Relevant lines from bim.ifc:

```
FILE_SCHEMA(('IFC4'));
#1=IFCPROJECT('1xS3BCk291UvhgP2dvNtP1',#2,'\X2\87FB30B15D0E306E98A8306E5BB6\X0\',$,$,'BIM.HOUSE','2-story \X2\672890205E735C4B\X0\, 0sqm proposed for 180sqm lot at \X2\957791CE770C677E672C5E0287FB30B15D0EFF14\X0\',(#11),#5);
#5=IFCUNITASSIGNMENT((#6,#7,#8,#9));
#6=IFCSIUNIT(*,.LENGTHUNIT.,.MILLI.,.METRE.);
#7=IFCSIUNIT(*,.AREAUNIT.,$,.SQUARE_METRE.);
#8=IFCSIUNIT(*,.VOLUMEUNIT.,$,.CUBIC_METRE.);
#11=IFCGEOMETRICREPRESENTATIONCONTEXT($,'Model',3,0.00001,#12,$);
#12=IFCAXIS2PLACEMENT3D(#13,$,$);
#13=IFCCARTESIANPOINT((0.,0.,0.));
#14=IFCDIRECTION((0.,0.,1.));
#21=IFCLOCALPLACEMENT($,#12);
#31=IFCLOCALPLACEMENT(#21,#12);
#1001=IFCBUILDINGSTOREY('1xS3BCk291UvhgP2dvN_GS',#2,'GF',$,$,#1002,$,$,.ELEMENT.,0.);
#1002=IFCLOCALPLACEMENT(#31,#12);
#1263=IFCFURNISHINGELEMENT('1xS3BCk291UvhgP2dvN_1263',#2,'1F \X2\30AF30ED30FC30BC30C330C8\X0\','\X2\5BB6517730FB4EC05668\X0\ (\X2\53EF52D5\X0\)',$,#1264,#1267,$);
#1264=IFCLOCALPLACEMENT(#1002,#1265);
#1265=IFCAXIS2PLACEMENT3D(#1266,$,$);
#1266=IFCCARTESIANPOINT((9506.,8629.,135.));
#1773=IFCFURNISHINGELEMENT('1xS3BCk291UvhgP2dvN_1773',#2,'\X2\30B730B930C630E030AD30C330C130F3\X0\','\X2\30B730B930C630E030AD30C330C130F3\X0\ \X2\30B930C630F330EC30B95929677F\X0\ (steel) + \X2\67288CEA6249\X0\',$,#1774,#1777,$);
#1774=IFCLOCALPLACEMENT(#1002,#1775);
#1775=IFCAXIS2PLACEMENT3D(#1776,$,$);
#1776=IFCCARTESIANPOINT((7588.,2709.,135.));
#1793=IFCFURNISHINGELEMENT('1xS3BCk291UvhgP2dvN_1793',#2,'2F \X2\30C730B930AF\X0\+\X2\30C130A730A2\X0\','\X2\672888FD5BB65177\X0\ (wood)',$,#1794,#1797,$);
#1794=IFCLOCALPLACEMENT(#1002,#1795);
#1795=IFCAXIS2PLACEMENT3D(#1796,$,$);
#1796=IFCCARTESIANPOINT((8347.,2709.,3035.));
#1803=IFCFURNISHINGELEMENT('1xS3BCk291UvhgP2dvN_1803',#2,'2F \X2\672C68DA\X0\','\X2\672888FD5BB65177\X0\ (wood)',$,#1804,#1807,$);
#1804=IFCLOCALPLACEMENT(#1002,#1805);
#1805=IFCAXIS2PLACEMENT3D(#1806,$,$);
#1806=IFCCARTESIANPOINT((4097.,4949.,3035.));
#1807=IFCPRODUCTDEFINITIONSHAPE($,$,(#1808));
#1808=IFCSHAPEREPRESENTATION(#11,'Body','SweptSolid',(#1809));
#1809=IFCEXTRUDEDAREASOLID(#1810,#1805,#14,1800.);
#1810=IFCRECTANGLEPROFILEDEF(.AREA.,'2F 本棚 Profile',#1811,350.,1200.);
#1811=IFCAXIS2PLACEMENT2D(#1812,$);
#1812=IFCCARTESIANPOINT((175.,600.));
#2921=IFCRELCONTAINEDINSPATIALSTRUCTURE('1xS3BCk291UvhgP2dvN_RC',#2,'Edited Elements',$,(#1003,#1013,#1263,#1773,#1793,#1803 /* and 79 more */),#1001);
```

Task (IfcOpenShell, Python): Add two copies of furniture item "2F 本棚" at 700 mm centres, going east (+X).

```python
import numpy as np
import ifcopenshell
import ifcopenshell.api.geometry
import ifcopenshell.api.root
import ifcopenshell.util.element
import ifcopenshell.util.placement
import ifcopenshell.util.unit

model = ifcopenshell.open("bim.ifc")
unit_scale = ifcopenshell.util.unit.calculate_unit_scale(model)


def reuse_history(source, copy):
    """copy_class also copies each property set's owner history, people and application; keep the originals."""
    for rel in copy.IsDefinedBy:
        if rel.is_a("IfcRelDefinesByProperties") and (history := rel.RelatingPropertyDefinition.OwnerHistory):
            rel.RelatingPropertyDefinition.OwnerHistory = source.OwnerHistory
            ifcopenshell.util.element.remove_deep2(model, history)


source = model.by_guid("1xS3BCk291UvhgP2dvN_1803")
base = ifcopenshell.util.placement.get_local_placement(source.ObjectPlacement)
step = np.array([1.0, 0.0, 0.0]) * 0.7 / unit_scale

for i in range(1, 3):
    copy = ifcopenshell.api.root.copy_class(model, product=source)
    copy.Representation = ifcopenshell.util.element.copy_deep(
        model, source.Representation, exclude=["IfcGeometricRepresentationContext", "IfcRepresentationMap"]
    )
    reuse_history(source, copy)
    matrix = base.copy()
    matrix[:3, 3] += i * step
    print("added at", matrix[:3, 3].round(3) + 0.0)
    ifcopenshell.api.geometry.edit_object_placement(model, product=copy, matrix=matrix, is_si=False)

model.write("bim_v2.ifc")
```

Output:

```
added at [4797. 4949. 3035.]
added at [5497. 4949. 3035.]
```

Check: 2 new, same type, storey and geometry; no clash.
